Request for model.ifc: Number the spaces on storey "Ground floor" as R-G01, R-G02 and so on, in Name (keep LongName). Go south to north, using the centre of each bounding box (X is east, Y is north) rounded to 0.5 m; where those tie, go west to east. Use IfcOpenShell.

First a look at what the model holds.

```python
import ifcopenshell
import ifcopenshell.util.element
import ifcopenshell.util.placement

model = ifcopenshell.open("model.ifc")
print(model.schema)
storey = next(s for s in model.by_type("IfcBuildingStorey") if s.Name == "Ground floor")
spaces = [e for e in ifcopenshell.util.element.get_decomposition(storey) if e.is_a("IfcSpace")]
for e in sorted(spaces, key=lambda e: e.id()):
    origin = ifcopenshell.util.placement.get_local_placement(e.ObjectPlacement)[:3, 3]
    print(e.id(), e.Name, e.LongName, origin.round(2) + 0.0, sep=" | ")
```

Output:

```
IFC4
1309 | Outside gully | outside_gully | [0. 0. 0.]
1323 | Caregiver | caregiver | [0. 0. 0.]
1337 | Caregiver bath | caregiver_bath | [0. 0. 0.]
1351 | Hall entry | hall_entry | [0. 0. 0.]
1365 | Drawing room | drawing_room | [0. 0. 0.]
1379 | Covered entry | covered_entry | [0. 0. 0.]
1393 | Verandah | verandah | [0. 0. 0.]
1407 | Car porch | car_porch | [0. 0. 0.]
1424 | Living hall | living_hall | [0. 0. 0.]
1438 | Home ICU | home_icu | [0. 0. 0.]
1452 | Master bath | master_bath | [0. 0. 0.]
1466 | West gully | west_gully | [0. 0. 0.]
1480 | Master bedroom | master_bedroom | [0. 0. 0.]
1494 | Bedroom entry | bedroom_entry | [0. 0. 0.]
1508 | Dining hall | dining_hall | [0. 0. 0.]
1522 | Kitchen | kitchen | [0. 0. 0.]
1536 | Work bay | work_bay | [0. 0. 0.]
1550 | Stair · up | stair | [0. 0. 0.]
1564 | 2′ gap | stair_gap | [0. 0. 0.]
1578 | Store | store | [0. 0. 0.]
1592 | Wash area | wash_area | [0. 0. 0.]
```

```python
import ifcopenshell
import ifcopenshell.geom
import ifcopenshell.util.element
import ifcopenshell.util.shape

model = ifcopenshell.open("model.ifc")
settings = ifcopenshell.geom.settings()
settings.set("use-world-coords", True)


def centre(element):
    shape = ifcopenshell.geom.create_shape(settings, element)
    return ifcopenshell.util.shape.get_bbox_centroid(shape.geometry)


storey = next(s for s in model.by_type("IfcBuildingStorey") if s.Name == "Ground floor")
spaces = [e for e in ifcopenshell.util.element.get_decomposition(storey) if e.is_a("IfcSpace")]

# Insertion points can sit at a corner or the storey origin, so sort by the geometry (in metres).
centres = {e: centre(e) for e in spaces}
spaces.sort(key=lambda e: (round(centres[e][1] / 0.5), centres[e][0]))

for i, e in enumerate(spaces, start=1):
    number = f"R-G{i:02d}"
    e.Name = number
    print(e.id(), number)

model.write("model_updated.ifc")
```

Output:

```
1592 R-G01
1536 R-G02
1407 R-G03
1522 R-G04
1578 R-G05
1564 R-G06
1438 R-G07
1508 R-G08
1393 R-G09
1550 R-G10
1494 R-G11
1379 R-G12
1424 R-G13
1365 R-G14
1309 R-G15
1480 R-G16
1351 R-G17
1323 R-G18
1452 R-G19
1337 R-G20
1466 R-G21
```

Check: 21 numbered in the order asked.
